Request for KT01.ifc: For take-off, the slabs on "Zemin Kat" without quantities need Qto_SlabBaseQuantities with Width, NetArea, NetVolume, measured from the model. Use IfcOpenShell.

First a look at what the model holds.

```python
import ifcopenshell
import ifcopenshell.util.element
import ifcopenshell.util.unit

model = ifcopenshell.open("KT01.ifc")
print(model.schema)
for unit_type in ("LENGTHUNIT", "AREAUNIT", "VOLUMEUNIT"):
    print(unit_type, ifcopenshell.util.unit.calculate_unit_scale(model, unit_type))
storey = next(s for s in model.by_type("IfcBuildingStorey") if s.Name == "Zemin Kat")
slabs = [e for e in ifcopenshell.util.element.get_decomposition(storey) if e.is_a("IfcSlab")]
for e in sorted(slabs, key=lambda e: e.id()):
    print(e.id(), e.is_a(), e.Name, list(ifcopenshell.util.element.get_psets(e, qtos_only=True)), sep=" | ")
```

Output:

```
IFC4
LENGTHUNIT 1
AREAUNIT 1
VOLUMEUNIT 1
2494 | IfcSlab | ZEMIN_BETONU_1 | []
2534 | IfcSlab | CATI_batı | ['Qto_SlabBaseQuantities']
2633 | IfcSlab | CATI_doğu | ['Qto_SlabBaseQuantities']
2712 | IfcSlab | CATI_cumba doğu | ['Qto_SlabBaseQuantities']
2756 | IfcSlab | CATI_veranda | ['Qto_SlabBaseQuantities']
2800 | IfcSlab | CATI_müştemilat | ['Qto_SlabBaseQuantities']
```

```python
import ifcopenshell
import ifcopenshell.api.pset
import ifcopenshell.geom
import ifcopenshell.util.element
import ifcopenshell.util.shape
import ifcopenshell.util.unit

model = ifcopenshell.open("KT01.ifc")
unit_scale = ifcopenshell.util.unit.calculate_unit_scale(model)
area_scale = ifcopenshell.util.unit.calculate_unit_scale(model, "AREAUNIT")
volume_scale = ifcopenshell.util.unit.calculate_unit_scale(model, "VOLUMEUNIT")
settings = ifcopenshell.geom.settings()

storey = next(s for s in model.by_type("IfcBuildingStorey") if s.Name == "Zemin Kat")
slabs = [e for e in ifcopenshell.util.element.get_decomposition(storey) if e.is_a("IfcSlab")]

for e in sorted(slabs, key=lambda e: e.id()):
    if ifcopenshell.util.element.get_psets(e, qtos_only=True, should_inherit=False):
        continue
    # Geometry comes back in metres, in the element's own axes.
    shape = ifcopenshell.geom.create_shape(settings, e)
    values = {
        "Width": ifcopenshell.util.shape.get_z(shape.geometry) / unit_scale,
        "NetArea": ifcopenshell.util.shape.get_footprint_area(shape.geometry) / area_scale,
        "NetVolume": ifcopenshell.util.shape.get_volume(shape.geometry) / volume_scale,
    }
    qto = ifcopenshell.api.pset.add_qto(model, product=e, name="Qto_SlabBaseQuantities")
    ifcopenshell.api.pset.edit_qto(model, qto=qto, properties=values)
    print(e.id(), {k: round(v, 3) for k, v in values.items()})

model.write("KT01_v2.ifc")
```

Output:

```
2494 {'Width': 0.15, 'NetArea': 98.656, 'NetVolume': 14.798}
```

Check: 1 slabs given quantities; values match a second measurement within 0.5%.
